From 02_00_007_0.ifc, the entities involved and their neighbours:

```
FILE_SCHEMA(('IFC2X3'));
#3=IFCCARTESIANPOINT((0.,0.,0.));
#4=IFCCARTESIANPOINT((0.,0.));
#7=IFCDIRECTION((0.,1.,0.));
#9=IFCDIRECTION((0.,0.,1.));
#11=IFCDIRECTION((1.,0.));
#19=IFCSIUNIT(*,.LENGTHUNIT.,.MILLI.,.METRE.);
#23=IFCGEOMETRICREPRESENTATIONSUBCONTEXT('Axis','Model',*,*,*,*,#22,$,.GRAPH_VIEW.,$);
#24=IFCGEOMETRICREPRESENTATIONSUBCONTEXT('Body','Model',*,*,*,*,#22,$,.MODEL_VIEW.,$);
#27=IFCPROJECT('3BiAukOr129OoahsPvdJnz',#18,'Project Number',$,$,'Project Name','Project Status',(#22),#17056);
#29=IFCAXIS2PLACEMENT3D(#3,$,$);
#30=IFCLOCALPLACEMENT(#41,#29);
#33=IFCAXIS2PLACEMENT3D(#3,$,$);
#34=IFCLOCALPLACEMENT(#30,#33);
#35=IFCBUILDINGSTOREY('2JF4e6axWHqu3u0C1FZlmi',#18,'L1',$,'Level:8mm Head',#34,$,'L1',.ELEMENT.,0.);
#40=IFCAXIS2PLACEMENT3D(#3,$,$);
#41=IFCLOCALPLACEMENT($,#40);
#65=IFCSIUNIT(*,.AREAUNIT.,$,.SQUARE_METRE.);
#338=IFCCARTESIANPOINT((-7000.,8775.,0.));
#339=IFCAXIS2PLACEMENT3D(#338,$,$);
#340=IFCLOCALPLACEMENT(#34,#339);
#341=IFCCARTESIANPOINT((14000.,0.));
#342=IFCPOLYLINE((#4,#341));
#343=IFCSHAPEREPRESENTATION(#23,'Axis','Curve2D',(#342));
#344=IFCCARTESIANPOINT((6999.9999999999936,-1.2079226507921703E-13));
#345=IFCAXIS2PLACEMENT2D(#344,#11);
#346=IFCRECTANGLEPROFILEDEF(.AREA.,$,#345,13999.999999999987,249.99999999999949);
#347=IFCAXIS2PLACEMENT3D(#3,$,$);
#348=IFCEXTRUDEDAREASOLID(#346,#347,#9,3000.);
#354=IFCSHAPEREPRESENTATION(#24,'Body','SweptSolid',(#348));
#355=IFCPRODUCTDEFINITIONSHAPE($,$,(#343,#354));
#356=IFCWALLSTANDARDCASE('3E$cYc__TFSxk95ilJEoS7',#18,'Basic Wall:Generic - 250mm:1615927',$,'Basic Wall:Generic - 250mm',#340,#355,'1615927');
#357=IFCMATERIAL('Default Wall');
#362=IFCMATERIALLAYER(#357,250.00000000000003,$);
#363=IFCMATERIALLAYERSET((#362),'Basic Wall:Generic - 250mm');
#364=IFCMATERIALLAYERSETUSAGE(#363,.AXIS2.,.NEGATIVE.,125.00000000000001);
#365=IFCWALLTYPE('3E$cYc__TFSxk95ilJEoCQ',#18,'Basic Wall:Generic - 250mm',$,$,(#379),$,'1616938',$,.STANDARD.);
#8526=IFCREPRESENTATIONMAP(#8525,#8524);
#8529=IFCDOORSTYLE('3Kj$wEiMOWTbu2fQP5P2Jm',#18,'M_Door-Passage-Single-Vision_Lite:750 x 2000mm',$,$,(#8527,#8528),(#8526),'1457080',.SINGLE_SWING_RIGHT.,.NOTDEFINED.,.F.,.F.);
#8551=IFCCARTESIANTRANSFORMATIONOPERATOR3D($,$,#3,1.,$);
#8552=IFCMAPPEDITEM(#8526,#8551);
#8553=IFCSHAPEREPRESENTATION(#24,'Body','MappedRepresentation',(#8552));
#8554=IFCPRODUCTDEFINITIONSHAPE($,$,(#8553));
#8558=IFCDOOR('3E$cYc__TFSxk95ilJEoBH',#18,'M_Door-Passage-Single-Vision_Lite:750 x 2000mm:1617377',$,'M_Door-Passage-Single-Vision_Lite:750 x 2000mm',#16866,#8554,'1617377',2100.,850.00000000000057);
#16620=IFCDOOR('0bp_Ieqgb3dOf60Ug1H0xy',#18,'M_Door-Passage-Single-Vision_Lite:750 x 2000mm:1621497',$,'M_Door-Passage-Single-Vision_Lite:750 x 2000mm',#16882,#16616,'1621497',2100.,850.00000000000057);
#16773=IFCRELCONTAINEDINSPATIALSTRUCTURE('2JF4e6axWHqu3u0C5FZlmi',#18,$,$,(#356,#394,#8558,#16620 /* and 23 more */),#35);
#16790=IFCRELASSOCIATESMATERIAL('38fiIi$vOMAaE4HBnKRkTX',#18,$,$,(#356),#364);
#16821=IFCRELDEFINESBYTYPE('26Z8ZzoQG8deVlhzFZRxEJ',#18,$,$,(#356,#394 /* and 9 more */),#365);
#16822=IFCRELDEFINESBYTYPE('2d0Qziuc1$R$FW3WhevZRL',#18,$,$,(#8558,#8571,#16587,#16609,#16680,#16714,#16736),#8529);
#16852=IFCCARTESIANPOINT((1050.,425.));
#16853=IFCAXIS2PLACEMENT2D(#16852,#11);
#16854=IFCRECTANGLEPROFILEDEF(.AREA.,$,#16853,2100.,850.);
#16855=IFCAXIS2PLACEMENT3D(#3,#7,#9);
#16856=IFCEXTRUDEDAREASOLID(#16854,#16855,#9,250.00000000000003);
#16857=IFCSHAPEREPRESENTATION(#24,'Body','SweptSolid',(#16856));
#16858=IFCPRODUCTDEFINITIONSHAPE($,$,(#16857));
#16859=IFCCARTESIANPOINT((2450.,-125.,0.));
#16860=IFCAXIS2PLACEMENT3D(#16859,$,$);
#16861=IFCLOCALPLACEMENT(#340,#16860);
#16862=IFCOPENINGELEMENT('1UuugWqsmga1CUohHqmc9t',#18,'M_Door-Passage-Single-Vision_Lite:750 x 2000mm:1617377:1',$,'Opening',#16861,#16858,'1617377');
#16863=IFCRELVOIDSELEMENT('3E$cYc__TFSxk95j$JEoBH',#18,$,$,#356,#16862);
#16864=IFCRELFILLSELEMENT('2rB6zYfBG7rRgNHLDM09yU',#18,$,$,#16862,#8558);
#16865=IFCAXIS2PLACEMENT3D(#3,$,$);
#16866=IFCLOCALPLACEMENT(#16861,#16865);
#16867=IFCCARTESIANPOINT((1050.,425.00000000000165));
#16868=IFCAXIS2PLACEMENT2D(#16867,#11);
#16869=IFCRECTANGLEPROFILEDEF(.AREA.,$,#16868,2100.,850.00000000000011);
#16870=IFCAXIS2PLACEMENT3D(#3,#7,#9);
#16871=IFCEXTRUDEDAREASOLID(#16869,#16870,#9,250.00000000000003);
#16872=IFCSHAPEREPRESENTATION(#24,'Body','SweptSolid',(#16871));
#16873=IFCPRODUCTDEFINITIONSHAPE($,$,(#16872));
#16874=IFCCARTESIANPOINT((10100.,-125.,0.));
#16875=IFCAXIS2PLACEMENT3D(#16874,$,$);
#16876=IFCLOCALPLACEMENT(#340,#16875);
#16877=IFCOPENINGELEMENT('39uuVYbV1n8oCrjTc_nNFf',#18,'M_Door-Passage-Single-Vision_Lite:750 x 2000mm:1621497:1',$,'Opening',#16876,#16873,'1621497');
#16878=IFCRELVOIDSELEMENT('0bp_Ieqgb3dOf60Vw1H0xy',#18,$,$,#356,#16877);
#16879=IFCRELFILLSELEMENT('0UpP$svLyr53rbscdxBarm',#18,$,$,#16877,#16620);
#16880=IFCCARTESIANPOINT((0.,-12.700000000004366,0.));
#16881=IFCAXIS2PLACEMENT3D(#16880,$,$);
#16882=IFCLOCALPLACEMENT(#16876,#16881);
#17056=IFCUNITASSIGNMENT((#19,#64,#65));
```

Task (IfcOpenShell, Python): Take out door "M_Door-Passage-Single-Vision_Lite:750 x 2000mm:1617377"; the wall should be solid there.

```python
import ifcopenshell
import ifcopenshell.api.feature
import ifcopenshell.api.root
import ifcopenshell.geom
import ifcopenshell.util.shape

model = ifcopenshell.open("02_00_007_0.ifc")
settings = ifcopenshell.geom.settings()


def volume(element):
    """Net volume in cubic metres, openings subtracted."""
    shape = ifcopenshell.geom.create_shape(settings, element)
    return ifcopenshell.util.shape.get_volume(shape.geometry)


door = model.by_guid("3E$cYc__TFSxk95ilJEoBH")
opening = door.FillsVoids[0].RelatingOpeningElement
wall = opening.VoidsElements[0].RelatingBuildingElement
before = volume(wall)

ifcopenshell.api.root.remove_product(model, product=door)
ifcopenshell.api.feature.remove_feature(model, feature=opening)

after = volume(wall)

print(f"wall volume {before:.3f} -> {after:.3f} m3")

model.write("02_00_007_0-out.ifc")
```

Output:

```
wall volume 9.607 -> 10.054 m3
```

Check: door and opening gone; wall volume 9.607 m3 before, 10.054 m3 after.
